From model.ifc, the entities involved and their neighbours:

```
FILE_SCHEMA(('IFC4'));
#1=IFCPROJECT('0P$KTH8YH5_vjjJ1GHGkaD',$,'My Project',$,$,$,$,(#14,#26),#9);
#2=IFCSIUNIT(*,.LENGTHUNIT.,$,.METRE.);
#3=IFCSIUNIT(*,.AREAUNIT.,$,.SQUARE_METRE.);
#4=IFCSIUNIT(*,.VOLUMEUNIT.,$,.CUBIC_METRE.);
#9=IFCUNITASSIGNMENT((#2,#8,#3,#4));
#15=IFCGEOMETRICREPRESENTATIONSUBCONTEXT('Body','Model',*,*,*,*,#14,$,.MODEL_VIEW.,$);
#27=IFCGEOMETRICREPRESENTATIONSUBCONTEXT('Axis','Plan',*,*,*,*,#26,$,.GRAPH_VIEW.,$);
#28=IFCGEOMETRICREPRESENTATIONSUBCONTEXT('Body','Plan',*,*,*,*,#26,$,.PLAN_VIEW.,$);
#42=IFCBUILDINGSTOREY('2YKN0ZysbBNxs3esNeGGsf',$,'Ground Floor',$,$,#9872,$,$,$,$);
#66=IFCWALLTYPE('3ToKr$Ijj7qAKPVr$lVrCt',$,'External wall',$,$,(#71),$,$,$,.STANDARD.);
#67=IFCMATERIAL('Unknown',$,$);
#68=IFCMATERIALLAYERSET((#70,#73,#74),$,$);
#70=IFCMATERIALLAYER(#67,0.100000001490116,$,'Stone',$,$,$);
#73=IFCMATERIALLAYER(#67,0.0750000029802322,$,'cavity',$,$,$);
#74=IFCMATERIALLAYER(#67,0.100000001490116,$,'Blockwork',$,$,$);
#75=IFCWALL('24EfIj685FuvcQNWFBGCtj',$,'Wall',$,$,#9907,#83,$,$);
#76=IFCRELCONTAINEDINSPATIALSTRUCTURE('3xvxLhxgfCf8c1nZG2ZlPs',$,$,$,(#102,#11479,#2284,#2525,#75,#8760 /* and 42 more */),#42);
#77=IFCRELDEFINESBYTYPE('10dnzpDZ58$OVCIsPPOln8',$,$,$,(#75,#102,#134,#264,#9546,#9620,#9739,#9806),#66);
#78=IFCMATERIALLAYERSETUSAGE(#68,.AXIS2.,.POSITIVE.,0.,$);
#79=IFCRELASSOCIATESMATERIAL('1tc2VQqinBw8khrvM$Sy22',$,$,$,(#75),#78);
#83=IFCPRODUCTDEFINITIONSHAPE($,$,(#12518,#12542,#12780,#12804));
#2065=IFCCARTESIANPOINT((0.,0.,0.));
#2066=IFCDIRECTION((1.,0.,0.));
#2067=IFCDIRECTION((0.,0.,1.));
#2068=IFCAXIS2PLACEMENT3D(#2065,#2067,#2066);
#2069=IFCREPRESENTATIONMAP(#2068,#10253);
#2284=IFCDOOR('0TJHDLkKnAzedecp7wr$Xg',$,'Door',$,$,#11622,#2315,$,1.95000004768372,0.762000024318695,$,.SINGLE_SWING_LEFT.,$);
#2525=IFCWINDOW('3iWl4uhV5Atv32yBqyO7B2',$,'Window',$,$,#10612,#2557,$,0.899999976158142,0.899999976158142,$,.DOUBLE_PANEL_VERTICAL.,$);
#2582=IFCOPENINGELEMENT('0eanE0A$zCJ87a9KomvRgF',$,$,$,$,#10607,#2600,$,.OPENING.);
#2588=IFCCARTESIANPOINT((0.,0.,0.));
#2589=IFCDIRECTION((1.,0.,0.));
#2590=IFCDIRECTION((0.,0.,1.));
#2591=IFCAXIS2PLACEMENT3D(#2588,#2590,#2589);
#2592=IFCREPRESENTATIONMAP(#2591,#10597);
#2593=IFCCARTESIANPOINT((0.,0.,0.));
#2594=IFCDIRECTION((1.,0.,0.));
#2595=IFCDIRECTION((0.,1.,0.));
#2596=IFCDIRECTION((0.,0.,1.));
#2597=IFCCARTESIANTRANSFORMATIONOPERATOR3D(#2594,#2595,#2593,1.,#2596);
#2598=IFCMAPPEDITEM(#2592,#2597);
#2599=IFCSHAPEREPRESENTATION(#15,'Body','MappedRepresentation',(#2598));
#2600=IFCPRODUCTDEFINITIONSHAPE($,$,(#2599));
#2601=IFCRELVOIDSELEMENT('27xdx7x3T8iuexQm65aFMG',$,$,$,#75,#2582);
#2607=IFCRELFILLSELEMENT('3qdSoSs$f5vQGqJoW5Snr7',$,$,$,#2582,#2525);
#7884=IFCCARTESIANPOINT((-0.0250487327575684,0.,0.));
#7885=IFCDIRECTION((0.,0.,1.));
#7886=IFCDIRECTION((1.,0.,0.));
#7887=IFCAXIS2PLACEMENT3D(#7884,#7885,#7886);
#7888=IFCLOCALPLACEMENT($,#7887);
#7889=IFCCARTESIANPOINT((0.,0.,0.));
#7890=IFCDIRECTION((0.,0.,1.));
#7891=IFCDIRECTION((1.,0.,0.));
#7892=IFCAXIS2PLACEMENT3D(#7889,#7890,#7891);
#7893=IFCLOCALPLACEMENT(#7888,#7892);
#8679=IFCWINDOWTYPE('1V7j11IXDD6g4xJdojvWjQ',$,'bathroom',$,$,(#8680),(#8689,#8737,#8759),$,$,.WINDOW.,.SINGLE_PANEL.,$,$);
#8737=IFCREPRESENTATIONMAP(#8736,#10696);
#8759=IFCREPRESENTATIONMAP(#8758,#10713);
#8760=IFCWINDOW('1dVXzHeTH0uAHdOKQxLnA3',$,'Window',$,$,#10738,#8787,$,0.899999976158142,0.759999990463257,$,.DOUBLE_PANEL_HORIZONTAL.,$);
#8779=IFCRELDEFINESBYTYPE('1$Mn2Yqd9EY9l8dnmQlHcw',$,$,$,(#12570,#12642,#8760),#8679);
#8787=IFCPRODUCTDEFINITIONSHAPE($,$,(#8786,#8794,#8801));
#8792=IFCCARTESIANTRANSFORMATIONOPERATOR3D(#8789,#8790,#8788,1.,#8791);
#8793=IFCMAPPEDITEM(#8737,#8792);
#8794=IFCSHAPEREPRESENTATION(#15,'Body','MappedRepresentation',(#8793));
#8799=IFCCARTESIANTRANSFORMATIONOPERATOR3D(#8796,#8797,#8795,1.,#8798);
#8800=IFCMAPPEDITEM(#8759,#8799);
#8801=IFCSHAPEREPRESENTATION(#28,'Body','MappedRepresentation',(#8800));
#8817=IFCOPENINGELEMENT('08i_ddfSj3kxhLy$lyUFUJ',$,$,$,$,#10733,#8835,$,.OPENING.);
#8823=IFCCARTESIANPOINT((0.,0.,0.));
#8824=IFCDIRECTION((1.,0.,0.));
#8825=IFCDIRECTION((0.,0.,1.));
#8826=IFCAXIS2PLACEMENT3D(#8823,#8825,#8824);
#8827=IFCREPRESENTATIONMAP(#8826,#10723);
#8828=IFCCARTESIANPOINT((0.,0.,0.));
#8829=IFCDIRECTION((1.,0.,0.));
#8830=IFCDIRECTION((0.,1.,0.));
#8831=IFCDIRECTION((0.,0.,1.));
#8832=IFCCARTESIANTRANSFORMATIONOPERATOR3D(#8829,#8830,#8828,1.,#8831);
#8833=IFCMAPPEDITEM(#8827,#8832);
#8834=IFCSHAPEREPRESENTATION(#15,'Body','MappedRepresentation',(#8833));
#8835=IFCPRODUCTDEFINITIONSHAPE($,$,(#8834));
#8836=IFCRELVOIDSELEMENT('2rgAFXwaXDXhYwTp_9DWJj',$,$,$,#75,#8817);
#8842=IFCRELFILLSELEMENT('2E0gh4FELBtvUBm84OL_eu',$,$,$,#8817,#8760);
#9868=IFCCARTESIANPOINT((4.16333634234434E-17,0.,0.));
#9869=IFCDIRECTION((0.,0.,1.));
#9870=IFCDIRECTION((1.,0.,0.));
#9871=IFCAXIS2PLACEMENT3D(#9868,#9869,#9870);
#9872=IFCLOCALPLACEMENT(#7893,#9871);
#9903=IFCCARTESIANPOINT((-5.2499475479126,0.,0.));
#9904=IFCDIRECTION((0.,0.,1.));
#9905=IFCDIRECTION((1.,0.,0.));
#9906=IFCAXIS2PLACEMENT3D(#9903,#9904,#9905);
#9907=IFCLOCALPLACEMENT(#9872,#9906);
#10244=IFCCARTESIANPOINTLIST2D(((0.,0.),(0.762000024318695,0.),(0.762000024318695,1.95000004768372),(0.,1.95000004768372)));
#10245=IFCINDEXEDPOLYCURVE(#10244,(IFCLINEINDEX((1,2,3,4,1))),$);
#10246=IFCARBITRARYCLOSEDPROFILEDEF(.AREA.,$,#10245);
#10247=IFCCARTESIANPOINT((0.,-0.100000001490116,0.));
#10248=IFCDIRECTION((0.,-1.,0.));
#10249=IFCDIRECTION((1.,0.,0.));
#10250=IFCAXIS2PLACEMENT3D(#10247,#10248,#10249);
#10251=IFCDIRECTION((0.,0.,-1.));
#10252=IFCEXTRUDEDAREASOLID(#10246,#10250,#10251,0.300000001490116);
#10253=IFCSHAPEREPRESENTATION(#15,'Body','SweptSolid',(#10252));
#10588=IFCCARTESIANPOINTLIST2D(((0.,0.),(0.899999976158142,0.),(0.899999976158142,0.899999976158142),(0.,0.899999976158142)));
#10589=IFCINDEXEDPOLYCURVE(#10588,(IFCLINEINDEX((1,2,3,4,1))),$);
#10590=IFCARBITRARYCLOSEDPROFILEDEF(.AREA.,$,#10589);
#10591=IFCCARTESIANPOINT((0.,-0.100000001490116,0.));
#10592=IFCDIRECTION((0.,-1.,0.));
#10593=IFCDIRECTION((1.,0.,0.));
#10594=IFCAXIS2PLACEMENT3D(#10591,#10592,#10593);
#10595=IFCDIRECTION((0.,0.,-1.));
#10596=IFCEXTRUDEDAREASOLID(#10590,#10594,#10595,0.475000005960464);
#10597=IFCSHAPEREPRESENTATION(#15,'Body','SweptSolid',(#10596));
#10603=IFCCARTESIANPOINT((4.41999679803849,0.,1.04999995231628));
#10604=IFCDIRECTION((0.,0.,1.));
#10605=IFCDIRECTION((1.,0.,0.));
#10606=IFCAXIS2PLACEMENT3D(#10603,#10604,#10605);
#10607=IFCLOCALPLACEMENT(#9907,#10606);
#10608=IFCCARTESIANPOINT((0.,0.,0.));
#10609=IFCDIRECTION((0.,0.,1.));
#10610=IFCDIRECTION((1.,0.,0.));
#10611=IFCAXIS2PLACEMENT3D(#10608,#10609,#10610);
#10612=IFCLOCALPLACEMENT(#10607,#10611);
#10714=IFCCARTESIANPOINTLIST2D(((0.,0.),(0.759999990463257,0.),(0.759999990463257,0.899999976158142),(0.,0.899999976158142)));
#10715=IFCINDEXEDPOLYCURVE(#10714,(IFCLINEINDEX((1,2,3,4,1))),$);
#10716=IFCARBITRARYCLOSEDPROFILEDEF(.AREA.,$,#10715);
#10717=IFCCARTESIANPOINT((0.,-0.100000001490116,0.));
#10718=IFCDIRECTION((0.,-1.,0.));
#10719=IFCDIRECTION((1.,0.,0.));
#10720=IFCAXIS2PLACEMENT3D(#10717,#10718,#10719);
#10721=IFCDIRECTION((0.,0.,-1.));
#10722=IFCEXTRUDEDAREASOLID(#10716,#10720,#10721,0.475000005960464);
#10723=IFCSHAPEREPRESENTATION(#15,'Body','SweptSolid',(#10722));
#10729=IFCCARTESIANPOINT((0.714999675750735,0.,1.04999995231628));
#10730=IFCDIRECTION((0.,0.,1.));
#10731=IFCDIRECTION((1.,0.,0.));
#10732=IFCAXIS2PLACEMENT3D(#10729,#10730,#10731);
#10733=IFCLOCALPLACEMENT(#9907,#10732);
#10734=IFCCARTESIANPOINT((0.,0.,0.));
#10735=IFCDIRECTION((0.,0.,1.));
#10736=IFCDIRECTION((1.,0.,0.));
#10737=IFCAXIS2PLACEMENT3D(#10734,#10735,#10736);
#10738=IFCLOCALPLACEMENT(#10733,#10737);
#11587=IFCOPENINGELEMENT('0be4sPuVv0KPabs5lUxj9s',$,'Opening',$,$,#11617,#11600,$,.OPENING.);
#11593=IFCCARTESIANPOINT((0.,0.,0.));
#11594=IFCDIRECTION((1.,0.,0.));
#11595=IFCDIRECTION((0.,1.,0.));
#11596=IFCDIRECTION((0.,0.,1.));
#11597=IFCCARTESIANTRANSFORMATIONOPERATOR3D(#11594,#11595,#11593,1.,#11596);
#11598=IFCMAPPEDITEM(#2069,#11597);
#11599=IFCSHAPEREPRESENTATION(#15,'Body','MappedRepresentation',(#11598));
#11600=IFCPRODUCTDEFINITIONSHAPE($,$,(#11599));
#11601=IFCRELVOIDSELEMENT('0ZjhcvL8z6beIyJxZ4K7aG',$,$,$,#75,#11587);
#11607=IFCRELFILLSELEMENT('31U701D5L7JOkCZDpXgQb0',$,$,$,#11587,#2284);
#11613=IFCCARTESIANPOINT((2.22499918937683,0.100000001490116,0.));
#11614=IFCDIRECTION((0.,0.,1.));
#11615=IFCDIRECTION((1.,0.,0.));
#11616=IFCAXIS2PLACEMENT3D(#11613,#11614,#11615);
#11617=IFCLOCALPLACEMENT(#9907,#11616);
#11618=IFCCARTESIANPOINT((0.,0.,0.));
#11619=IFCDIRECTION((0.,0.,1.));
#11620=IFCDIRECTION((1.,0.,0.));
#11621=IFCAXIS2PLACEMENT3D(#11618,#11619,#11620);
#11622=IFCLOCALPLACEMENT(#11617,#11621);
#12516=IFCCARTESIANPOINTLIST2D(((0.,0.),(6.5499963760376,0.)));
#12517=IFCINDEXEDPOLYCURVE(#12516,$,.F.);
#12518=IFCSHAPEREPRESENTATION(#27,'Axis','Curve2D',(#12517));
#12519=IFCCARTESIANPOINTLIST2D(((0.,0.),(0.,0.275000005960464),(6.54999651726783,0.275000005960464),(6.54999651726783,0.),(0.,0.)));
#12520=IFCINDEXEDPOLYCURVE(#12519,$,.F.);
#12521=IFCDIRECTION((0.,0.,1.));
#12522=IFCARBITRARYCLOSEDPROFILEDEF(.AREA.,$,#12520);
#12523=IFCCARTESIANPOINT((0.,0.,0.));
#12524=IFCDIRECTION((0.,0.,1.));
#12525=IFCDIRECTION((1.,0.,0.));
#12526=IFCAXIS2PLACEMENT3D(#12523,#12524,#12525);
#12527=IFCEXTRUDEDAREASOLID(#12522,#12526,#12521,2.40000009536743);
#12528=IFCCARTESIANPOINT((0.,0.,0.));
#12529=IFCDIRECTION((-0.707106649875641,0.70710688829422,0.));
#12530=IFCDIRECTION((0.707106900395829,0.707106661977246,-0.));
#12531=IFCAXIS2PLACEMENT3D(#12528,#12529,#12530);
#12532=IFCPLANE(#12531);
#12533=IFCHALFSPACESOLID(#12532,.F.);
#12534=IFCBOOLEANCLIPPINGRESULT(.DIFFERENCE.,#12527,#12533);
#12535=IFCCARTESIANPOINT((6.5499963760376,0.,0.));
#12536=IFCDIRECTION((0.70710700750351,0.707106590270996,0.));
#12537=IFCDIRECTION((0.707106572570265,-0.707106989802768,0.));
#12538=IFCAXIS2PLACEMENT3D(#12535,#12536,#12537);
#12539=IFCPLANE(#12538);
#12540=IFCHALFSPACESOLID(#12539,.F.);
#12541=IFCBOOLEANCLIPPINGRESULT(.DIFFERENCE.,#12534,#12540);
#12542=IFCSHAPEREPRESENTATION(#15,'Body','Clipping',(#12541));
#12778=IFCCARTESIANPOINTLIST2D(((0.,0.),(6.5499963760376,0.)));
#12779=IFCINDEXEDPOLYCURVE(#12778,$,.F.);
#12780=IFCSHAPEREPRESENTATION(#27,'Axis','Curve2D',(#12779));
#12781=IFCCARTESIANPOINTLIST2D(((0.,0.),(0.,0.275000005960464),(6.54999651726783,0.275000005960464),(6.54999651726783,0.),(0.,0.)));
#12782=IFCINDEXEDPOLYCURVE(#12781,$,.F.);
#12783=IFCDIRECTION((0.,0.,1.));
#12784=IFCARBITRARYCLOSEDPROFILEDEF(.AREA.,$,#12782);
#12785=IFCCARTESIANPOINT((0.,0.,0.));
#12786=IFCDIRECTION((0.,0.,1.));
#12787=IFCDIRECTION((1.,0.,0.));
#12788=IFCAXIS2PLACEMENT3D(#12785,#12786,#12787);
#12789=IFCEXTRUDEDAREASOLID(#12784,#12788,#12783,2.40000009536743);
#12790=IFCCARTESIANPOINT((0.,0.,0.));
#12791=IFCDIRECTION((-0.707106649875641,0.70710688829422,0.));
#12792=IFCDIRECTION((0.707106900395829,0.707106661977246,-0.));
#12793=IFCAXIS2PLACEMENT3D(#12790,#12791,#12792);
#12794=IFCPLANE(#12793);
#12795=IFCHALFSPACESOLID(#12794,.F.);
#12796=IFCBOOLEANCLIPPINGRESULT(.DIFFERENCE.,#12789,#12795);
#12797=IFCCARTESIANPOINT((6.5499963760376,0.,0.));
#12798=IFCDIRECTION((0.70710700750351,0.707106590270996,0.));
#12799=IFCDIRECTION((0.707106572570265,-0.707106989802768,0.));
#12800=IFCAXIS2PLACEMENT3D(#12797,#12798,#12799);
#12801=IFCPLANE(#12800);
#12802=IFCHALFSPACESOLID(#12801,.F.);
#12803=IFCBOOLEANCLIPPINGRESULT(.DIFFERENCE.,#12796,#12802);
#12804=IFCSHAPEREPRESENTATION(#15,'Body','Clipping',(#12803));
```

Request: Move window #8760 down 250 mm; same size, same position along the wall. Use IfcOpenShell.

```python
import numpy as np
import ifcopenshell
import ifcopenshell.api.geometry
import ifcopenshell.util.placement
import ifcopenshell.util.unit

model = ifcopenshell.open("model.ifc")
unit_scale = ifcopenshell.util.unit.calculate_unit_scale(model)

window = model.by_guid("1dVXzHeTH0uAHdOKQxLnA3")
opening = window.FillsVoids[0].RelatingOpeningElement
dz = -0.25 / unit_scale

shift = np.array([0.0, 0.0, dz])
# The window is placed relative to its opening, so it follows when the opening moves.
matrix = ifcopenshell.util.placement.get_local_placement(opening.ObjectPlacement)
matrix[:3, 3] += shift
ifcopenshell.api.geometry.edit_object_placement(
    model, product=opening, matrix=matrix, is_si=False, should_transform_children=True
)

print(f"moved by {dz * unit_scale:+.3f} m")

model.write("model_edited.ifc")
```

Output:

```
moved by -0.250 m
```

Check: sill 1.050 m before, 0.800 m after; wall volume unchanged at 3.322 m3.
